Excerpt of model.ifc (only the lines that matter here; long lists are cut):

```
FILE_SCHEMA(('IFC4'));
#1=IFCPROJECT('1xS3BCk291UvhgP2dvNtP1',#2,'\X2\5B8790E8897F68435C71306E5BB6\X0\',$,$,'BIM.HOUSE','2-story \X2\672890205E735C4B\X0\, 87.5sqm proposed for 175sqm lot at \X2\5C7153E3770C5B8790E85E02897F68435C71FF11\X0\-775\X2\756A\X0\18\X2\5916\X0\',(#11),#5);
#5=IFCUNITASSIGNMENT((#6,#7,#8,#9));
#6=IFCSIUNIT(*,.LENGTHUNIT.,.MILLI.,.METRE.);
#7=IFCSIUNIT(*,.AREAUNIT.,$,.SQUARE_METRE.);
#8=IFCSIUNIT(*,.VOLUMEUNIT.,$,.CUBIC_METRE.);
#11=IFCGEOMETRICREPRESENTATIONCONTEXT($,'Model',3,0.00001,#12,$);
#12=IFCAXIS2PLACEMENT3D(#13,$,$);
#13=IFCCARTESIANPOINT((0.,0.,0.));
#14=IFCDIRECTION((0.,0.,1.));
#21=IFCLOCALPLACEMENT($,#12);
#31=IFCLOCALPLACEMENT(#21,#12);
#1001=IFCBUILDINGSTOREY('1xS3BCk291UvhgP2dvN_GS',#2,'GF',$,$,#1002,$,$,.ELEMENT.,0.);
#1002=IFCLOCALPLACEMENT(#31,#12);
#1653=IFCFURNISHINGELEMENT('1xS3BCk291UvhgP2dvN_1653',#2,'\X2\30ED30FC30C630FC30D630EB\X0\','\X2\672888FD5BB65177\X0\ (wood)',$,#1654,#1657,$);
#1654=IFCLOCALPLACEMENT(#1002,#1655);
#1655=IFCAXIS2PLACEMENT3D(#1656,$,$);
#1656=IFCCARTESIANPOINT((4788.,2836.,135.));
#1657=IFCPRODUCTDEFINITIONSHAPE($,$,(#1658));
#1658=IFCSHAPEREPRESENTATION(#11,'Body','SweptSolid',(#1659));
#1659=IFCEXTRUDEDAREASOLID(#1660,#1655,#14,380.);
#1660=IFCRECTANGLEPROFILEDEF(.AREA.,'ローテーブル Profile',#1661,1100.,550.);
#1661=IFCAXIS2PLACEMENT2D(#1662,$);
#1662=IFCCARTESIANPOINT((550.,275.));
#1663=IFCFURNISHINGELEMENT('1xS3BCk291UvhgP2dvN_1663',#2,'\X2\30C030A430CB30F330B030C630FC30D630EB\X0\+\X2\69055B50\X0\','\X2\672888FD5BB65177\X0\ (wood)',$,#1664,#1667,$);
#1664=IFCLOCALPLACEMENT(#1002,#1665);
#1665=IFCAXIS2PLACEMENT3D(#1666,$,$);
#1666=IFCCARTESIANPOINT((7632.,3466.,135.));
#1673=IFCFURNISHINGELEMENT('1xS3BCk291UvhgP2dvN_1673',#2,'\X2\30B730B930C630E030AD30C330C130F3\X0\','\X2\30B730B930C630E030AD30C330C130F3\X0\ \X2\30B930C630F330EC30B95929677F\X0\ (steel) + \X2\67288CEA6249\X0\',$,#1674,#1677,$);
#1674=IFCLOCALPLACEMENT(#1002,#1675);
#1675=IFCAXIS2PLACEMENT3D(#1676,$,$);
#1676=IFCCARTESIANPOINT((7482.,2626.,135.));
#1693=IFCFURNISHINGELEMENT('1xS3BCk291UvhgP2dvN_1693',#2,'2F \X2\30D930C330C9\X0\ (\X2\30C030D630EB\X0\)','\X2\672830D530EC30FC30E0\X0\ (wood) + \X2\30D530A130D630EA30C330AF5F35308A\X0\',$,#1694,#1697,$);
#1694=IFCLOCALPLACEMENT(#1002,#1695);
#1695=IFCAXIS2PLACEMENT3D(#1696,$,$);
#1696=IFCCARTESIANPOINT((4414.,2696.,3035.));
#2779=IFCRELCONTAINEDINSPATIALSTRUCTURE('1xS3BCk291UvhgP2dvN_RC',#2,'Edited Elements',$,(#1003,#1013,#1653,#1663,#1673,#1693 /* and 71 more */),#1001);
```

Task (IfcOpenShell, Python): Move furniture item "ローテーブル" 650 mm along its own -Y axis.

```python
import ifcopenshell
import ifcopenshell.api.geometry
import ifcopenshell.util.placement

model = ifcopenshell.open("model.ifc")

item = model.by_id(1653)
matrix = ifcopenshell.util.placement.get_local_placement(item.ObjectPlacement)
matrix[:3, 3] -= matrix[:3, 1] * 650.0
ifcopenshell.api.geometry.edit_object_placement(model, product=item, matrix=matrix, is_si=False)

print(ifcopenshell.util.placement.get_local_placement(item.ObjectPlacement).round(3) + 0.0)

model.write("model_edited.ifc")
```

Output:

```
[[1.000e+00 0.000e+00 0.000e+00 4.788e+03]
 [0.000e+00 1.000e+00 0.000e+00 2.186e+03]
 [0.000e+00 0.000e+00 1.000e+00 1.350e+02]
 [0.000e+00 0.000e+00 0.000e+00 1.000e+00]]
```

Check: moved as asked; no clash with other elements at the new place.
